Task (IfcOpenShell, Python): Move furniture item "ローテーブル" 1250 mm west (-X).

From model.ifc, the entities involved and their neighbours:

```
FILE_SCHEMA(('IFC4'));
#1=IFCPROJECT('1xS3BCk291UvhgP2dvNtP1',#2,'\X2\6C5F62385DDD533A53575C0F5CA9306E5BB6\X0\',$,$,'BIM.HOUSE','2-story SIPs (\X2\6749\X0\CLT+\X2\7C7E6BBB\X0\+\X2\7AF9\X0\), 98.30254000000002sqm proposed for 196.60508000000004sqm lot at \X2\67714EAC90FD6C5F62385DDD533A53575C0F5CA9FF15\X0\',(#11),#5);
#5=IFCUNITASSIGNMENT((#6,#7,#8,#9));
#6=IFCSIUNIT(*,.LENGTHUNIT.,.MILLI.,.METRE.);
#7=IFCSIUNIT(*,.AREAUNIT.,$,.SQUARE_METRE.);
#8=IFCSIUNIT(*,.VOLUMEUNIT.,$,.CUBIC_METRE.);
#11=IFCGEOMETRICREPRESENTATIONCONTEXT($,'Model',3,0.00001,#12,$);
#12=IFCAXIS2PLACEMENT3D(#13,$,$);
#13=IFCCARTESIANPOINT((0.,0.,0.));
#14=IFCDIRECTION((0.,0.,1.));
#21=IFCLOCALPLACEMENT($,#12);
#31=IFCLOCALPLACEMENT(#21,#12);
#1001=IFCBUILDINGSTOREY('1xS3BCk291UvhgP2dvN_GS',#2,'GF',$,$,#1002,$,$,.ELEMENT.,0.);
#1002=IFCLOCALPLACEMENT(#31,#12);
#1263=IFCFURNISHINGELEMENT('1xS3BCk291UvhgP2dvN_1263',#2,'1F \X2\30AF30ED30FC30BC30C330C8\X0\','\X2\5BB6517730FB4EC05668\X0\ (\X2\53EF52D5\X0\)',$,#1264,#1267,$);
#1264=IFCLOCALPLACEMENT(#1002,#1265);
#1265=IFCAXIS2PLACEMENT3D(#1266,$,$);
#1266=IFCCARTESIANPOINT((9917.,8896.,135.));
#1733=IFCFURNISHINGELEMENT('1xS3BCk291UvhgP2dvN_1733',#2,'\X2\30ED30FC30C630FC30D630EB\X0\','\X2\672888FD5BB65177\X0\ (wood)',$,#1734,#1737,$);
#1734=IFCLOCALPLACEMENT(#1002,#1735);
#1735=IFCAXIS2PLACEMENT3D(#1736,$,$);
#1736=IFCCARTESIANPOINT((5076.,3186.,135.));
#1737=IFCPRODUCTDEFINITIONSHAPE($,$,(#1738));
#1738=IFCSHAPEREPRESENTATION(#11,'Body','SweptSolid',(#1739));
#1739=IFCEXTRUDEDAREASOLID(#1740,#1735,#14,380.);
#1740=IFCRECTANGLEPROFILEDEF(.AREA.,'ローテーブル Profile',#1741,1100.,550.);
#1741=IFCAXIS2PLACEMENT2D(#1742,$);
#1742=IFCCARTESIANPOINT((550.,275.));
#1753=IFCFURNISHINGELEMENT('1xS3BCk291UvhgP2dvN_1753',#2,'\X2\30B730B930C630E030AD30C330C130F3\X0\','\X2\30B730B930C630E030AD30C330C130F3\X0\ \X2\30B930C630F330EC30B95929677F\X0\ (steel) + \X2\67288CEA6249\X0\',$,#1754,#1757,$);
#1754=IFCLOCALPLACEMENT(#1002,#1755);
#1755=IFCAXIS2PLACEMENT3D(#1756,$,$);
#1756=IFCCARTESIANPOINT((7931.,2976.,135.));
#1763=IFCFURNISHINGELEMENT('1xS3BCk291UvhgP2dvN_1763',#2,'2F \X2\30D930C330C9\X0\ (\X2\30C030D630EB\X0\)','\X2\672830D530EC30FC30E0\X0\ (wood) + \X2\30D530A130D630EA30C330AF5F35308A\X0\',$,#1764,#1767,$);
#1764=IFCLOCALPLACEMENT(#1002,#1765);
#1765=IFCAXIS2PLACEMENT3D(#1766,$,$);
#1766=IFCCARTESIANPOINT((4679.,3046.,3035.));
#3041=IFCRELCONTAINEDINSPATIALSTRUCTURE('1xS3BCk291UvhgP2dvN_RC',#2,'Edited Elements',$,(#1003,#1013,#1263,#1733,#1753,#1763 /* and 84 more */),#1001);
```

```python
import ifcopenshell
import ifcopenshell.api.geometry
import ifcopenshell.util.placement
import ifcopenshell.util.unit

model = ifcopenshell.open("model.ifc")
unit_scale = ifcopenshell.util.unit.calculate_unit_scale(model)

item = model.by_id(1733)
matrix = ifcopenshell.util.placement.get_local_placement(item.ObjectPlacement)
matrix[0, 3] -= 1.25 / unit_scale
ifcopenshell.api.geometry.edit_object_placement(model, product=item, matrix=matrix, is_si=False)

print(ifcopenshell.util.placement.get_local_placement(item.ObjectPlacement).round(3) + 0.0)

model.write("model_v2.ifc")
```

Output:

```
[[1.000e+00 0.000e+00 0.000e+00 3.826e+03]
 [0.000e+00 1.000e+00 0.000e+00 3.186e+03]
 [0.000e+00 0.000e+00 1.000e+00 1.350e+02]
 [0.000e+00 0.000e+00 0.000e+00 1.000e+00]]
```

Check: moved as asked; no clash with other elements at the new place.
